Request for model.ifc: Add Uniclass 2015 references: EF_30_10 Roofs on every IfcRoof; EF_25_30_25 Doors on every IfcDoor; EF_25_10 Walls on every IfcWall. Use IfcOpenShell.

First a look at what the model holds.

```python
import ifcopenshell

model = ifcopenshell.open("model.ifc")
print(model.schema)
print("classifications:", [c.Name for c in model.by_type("IfcClassification")])
for ifc_class in ("IfcDoor", "IfcRoof", "IfcStair", "IfcWall", "IfcWindow"):
    print(ifc_class, len(model.by_type(ifc_class)))
```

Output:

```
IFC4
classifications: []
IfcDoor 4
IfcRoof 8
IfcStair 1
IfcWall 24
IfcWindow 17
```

```python
import ifcopenshell
import ifcopenshell.api.classification

model = ifcopenshell.open("model.ifc")

system = ifcopenshell.api.classification.add_classification(model, classification="Uniclass 2015")

codes = {
    "IfcRoof": ("EF_30_10", "Roofs"),
    "IfcDoor": ("EF_25_30_25", "Doors"),
    "IfcWall": ("EF_25_10", "Walls"),
}
for ifc_class, (code, name) in codes.items():
    products = model.by_type(ifc_class)
    ifcopenshell.api.classification.add_reference(
        model, products=products, classification=system, identification=code, name=name
    )
    print(code, len(products))

model.write("model-out.ifc")
```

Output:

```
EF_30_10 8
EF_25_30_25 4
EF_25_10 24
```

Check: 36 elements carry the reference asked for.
